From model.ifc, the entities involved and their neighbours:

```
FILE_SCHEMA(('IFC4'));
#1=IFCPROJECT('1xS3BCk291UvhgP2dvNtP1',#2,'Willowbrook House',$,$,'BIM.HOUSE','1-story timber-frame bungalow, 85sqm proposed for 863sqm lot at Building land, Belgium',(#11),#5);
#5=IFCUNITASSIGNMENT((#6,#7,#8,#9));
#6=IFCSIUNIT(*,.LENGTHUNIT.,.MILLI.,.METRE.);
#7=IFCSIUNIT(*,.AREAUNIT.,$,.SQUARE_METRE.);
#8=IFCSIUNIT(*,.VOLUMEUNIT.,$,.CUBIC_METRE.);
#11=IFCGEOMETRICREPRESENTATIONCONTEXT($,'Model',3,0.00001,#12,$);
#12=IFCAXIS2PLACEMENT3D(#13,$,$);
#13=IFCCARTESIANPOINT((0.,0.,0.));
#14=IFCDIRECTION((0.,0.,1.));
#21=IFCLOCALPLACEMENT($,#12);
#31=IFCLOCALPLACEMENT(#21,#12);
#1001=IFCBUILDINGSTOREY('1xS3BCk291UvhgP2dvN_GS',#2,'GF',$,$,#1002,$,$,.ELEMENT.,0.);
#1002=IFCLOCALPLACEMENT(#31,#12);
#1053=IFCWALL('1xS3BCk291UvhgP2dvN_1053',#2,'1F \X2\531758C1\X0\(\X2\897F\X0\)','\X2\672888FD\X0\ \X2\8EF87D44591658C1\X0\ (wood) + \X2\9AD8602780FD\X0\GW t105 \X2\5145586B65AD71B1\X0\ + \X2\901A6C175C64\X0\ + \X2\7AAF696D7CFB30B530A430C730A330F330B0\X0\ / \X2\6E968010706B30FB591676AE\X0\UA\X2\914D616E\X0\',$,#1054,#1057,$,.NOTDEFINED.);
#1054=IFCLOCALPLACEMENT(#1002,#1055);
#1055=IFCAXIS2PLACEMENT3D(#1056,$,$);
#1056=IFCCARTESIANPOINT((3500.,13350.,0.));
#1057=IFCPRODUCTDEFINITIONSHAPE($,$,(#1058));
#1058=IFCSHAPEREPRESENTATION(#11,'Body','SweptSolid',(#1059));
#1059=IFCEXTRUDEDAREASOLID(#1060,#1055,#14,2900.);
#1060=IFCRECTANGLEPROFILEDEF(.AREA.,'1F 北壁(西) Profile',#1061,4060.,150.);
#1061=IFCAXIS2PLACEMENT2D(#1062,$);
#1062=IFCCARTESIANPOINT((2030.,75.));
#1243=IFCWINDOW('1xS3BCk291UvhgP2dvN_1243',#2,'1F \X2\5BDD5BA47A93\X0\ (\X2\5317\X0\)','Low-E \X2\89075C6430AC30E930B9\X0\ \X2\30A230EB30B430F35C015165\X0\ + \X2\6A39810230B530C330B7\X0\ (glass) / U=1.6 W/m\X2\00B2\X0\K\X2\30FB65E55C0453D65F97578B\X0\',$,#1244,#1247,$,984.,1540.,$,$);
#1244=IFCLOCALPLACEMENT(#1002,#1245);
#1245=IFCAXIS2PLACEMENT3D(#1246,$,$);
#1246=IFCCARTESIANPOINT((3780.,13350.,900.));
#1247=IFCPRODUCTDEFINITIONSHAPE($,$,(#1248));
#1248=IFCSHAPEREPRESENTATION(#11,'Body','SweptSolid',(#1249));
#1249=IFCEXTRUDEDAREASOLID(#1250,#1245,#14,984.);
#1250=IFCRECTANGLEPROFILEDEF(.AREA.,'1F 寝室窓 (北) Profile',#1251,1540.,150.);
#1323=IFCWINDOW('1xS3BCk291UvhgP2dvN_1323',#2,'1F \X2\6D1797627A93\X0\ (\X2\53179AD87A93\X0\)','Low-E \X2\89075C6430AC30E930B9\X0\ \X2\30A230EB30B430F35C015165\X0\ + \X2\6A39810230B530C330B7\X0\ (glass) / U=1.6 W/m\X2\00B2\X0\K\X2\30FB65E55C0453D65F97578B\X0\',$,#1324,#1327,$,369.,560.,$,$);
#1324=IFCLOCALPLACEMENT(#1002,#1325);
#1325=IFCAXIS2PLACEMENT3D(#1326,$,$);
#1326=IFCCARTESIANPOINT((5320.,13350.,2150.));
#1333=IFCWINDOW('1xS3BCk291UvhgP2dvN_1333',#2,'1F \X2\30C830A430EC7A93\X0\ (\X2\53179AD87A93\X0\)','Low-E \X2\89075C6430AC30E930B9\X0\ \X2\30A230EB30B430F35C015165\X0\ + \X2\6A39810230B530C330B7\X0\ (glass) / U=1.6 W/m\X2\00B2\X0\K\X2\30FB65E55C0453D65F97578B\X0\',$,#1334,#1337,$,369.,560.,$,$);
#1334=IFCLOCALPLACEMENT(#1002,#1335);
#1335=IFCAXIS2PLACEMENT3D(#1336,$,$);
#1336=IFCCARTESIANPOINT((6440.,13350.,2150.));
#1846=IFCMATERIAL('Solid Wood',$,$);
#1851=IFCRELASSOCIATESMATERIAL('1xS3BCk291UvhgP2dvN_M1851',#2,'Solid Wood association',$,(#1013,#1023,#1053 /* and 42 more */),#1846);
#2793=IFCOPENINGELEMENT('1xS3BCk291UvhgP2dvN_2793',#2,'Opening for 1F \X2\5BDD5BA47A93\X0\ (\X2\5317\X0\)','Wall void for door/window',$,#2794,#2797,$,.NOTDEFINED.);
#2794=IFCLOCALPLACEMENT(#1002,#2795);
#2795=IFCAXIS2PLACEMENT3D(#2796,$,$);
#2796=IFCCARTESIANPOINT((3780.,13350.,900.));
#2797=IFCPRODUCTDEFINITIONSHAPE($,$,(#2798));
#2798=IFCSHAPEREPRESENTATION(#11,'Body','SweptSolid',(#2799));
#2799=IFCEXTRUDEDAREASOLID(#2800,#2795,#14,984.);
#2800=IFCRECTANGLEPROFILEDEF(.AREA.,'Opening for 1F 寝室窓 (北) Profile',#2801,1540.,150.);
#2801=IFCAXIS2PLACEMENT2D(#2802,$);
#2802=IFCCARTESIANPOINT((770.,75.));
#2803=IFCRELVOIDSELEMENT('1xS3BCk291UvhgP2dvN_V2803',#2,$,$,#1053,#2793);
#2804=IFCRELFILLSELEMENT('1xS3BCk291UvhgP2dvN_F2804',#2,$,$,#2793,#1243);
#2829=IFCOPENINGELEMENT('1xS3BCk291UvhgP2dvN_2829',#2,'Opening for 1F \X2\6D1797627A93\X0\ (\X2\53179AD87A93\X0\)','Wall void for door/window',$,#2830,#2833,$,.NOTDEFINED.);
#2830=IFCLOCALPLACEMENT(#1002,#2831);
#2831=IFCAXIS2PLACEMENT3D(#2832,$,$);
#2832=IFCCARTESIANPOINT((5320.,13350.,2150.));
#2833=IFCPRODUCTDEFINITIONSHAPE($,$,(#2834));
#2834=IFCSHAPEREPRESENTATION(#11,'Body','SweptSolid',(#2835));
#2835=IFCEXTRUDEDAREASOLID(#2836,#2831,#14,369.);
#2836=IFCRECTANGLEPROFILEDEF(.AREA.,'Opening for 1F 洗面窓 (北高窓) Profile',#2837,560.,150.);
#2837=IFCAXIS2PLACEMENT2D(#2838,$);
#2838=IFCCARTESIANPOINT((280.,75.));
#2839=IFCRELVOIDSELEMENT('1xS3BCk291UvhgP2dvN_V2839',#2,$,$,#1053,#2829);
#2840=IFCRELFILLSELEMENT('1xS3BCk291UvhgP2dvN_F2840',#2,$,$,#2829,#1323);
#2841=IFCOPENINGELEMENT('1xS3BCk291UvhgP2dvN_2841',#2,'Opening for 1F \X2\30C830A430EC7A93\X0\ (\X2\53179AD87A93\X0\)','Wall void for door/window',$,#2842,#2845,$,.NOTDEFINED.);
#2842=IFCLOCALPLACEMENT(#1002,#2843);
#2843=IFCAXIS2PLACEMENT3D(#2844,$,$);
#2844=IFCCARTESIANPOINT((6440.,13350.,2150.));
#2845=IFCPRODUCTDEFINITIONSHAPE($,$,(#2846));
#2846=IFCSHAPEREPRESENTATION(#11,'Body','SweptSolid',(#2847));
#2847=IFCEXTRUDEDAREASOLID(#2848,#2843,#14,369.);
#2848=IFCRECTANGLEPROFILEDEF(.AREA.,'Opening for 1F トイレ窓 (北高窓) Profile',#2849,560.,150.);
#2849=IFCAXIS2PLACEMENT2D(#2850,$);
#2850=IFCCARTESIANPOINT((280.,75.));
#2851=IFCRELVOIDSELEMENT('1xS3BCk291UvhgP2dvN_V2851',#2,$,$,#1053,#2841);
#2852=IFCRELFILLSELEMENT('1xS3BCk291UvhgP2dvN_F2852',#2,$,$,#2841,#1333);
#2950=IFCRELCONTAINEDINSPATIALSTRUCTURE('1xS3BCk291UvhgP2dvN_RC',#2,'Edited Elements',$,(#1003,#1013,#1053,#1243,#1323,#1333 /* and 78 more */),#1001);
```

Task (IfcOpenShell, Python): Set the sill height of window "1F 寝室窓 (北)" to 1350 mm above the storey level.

```python
import numpy as np
import ifcopenshell
import ifcopenshell.api.geometry
import ifcopenshell.geom
import ifcopenshell.util.element
import ifcopenshell.util.placement
import ifcopenshell.util.shape
import ifcopenshell.util.unit

model = ifcopenshell.open("model.ifc")
unit_scale = ifcopenshell.util.unit.calculate_unit_scale(model)

window = model.by_id(1243)
opening = window.FillsVoids[0].RelatingOpeningElement
storey = ifcopenshell.util.element.get_container(window, ifc_class="IfcBuildingStorey")
level = ifcopenshell.util.placement.get_local_placement(storey.ObjectPlacement)[2, 3]

# The opening's origin need not be at the sill, so measure its lowest point.
shape = ifcopenshell.geom.create_shape(ifcopenshell.geom.settings(), opening)
bottom = ifcopenshell.util.shape.get_shape_bottom_elevation(shape, shape.geometry) / unit_scale
dz = level + 1.35 / unit_scale - bottom

shift = np.array([0.0, 0.0, dz])
# The window is not placed relative to its opening, so move both.
for product in (opening, window):
    matrix = ifcopenshell.util.placement.get_local_placement(product.ObjectPlacement)
    matrix[:3, 3] += shift
    ifcopenshell.api.geometry.edit_object_placement(model, product=product, matrix=matrix, is_si=False)

print(f"moved by {dz * unit_scale:+.3f} m")

model.write("model_edited.ifc")
```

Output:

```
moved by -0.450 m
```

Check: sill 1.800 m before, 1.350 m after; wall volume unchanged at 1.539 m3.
